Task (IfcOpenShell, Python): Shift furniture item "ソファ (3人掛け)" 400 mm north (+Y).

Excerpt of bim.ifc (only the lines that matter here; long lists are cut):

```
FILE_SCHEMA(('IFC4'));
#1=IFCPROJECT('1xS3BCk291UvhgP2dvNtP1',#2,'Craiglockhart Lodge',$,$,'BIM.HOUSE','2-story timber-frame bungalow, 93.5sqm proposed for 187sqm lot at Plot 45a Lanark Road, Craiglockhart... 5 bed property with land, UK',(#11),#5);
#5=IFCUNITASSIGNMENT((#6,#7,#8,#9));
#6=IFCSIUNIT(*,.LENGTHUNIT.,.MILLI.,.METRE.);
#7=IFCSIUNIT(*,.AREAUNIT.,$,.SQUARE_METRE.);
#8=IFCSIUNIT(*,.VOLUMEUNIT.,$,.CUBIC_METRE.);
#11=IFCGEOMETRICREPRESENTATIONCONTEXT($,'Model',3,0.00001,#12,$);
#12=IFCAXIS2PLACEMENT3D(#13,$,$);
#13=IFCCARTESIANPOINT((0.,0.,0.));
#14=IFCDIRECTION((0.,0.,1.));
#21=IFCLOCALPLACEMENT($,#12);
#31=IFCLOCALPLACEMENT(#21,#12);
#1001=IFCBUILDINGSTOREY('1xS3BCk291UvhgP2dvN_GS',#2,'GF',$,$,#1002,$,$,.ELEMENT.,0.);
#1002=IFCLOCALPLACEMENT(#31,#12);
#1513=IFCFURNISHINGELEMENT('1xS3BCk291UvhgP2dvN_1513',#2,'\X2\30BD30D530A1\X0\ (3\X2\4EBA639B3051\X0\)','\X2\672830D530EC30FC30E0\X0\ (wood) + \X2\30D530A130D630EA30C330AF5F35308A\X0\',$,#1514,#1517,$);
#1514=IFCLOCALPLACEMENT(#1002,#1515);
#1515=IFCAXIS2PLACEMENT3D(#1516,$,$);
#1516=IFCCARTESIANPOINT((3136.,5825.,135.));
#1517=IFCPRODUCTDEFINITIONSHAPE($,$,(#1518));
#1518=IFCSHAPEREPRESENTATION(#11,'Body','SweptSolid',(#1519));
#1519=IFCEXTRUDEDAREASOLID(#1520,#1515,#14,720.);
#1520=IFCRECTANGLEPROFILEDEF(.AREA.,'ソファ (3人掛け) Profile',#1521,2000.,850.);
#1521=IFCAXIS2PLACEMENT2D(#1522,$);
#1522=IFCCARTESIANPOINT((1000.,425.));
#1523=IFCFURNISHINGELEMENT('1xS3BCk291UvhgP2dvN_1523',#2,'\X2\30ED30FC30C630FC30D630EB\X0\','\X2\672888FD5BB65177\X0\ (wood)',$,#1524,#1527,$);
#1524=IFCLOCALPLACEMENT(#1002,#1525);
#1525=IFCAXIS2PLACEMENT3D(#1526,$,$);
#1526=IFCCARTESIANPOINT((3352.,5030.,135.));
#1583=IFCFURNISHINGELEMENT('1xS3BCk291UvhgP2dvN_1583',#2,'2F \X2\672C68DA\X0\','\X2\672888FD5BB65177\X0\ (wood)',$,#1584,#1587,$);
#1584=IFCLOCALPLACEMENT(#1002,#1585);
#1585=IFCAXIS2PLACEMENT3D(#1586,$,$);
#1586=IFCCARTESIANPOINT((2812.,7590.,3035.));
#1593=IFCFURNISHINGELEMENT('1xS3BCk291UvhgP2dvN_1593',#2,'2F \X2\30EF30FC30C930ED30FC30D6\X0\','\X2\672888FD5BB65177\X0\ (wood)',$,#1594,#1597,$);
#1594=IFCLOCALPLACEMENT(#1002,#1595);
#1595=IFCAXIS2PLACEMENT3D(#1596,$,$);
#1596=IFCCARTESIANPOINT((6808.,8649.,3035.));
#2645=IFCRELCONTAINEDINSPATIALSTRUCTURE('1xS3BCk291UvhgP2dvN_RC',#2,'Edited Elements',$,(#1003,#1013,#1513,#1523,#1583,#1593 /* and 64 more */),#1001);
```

```python
import ifcopenshell
import ifcopenshell.api.geometry
import ifcopenshell.util.placement
import ifcopenshell.util.unit

model = ifcopenshell.open("bim.ifc")
unit_scale = ifcopenshell.util.unit.calculate_unit_scale(model)

item = model.by_id(1513)
matrix = ifcopenshell.util.placement.get_local_placement(item.ObjectPlacement)
matrix[1, 3] += 0.4 / unit_scale
ifcopenshell.api.geometry.edit_object_placement(model, product=item, matrix=matrix, is_si=False)

print(ifcopenshell.util.placement.get_local_placement(item.ObjectPlacement).round(3) + 0.0)

model.write("bim-out.ifc")
```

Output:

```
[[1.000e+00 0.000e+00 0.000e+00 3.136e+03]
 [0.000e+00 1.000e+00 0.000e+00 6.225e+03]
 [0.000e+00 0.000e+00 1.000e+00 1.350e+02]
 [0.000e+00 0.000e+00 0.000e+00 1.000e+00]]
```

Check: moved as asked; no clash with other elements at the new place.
